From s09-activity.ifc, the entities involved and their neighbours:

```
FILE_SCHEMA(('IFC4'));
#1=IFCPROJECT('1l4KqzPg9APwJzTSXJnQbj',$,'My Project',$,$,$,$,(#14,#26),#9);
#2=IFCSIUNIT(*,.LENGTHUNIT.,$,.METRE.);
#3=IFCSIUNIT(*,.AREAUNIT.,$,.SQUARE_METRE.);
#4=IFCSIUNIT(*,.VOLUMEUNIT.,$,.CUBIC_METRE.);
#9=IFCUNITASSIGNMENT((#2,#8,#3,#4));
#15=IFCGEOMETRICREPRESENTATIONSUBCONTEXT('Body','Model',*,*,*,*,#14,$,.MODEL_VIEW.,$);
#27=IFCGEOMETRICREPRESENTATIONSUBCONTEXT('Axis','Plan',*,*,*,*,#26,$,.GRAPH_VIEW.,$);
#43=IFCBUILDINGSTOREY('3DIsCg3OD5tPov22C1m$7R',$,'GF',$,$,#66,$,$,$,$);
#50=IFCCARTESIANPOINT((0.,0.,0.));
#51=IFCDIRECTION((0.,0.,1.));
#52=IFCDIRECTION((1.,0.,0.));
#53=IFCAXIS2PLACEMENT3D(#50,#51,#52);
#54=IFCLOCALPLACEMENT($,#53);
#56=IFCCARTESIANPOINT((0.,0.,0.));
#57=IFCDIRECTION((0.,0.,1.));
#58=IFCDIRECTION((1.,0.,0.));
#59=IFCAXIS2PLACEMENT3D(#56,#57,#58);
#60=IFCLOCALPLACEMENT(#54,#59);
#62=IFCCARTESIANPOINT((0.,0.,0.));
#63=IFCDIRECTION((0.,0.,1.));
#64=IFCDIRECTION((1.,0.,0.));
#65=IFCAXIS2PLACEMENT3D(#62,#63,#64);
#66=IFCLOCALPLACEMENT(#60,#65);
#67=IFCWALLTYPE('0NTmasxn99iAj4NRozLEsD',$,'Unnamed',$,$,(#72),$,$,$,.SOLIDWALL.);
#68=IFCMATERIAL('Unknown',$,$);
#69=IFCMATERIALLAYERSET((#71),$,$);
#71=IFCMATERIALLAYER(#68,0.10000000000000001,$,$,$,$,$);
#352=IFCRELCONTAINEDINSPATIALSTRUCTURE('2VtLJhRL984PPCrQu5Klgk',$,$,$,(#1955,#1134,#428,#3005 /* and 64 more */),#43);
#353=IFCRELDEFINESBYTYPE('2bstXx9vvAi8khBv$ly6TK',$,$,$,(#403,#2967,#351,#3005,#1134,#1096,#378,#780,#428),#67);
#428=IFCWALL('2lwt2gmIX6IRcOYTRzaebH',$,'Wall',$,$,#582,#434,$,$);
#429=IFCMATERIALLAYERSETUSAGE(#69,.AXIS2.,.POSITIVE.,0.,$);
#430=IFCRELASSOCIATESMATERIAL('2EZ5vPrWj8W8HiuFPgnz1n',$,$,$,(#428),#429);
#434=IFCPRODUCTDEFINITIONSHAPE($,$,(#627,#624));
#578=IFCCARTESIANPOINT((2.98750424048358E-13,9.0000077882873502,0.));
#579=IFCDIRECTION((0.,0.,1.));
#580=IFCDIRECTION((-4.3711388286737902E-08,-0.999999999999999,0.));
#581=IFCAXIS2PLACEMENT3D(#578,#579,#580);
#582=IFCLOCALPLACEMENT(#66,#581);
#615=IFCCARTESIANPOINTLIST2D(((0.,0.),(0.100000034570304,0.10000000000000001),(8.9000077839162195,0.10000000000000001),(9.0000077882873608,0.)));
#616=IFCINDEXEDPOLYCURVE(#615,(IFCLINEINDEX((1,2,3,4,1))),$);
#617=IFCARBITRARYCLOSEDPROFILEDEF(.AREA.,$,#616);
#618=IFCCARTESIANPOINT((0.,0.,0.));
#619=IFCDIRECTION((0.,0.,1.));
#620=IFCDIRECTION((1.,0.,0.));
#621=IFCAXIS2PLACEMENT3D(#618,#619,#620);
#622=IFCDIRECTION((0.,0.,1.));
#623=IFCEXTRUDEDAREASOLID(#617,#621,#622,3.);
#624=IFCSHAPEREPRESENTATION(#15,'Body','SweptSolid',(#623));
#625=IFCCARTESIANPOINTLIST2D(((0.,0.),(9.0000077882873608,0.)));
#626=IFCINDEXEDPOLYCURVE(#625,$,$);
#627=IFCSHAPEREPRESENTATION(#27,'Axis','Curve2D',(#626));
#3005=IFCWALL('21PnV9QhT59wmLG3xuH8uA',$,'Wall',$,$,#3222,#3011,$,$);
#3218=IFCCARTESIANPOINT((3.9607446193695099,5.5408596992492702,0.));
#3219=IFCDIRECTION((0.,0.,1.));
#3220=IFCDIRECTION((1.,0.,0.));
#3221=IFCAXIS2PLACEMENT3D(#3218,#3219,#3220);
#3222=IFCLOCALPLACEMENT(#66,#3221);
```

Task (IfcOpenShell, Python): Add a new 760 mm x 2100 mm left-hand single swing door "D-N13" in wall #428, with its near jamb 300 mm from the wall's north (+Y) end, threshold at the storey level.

```python
import numpy as np
import ifcopenshell
import ifcopenshell.api.feature
import ifcopenshell.api.geometry
import ifcopenshell.api.root
import ifcopenshell.api.spatial
import ifcopenshell.geom
import ifcopenshell.util.element
import ifcopenshell.util.placement
import ifcopenshell.util.representation
import ifcopenshell.util.shape
import ifcopenshell.util.unit

model = ifcopenshell.open("s09-activity.ifc")
unit_scale = ifcopenshell.util.unit.calculate_unit_scale(model)
settings = ifcopenshell.geom.settings()


def volume(element):
    """Net volume in cubic metres, openings subtracted."""
    shape = ifcopenshell.geom.create_shape(settings, element)
    return ifcopenshell.util.shape.get_volume(shape.geometry)


wall = model.by_guid("2lwt2gmIX6IRcOYTRzaebH")
storey = ifcopenshell.util.element.get_container(wall, ifc_class="IfcBuildingStorey")
context = ifcopenshell.util.representation.get_context(model, "Model", "Body", "MODEL_VIEW")
before = volume(wall)

width, height, from_end, sill = 0.76, 2.1, 0.3, 0.0  # metres

# The wall runs along its own X axis, and the end named is its -X end.
wall_shape = ifcopenshell.geom.create_shape(settings, wall)
x, y, z = ifcopenshell.util.shape.get_vertices(wall_shape.geometry).T
start = x.min() + from_end
face, thickness = float(y.min()), float(y.max() - y.min())
wall_matrix = ifcopenshell.util.placement.get_local_placement(wall.ObjectPlacement)
level = ifcopenshell.util.placement.get_local_placement(storey.ObjectPlacement)[2, 3]


def in_wall(x, y):
    """Placement at x, y metres in the wall's axes, at sill height."""
    matrix = wall_matrix.copy()
    matrix[:, 3] = wall_matrix @ np.array([x / unit_scale, y / unit_scale, 0.0, 1.0])
    matrix[2, 3] = level + sill / unit_scale
    return matrix


# Opening: a box that overshoots both wall faces by 50 mm.
opening = ifcopenshell.api.root.create_entity(model, ifc_class="IfcOpeningElement", predefined_type="OPENING")
box = ifcopenshell.api.geometry.add_wall_representation(
    model, context=context, length=width, height=height, thickness=thickness + 0.1
)
ifcopenshell.api.geometry.assign_representation(model, product=opening, representation=box)
ifcopenshell.api.geometry.edit_object_placement(model, product=opening, matrix=in_wall(start, face - 0.05), is_si=False)
ifcopenshell.api.feature.add_feature(model, feature=opening, element=wall)

door = ifcopenshell.api.root.create_entity(model, ifc_class="IfcDoor", name="D-N13", predefined_type="DOOR")
door.OverallWidth, door.OverallHeight = width / unit_scale, height / unit_scale
door.OperationType = "SINGLE_SWING_LEFT"
body = ifcopenshell.api.geometry.add_door_representation(
    model,
    context=context,
    overall_width=door.OverallWidth,
    overall_height=door.OverallHeight,
    operation_type="SINGLE_SWING_LEFT",
    lining_properties={"LiningDepth": thickness / unit_scale, "ThresholdDepth": thickness / unit_scale},
)
ifcopenshell.api.geometry.assign_representation(model, product=door, representation=body)
ifcopenshell.api.spatial.assign_container(model, products=[door], relating_structure=storey)
ifcopenshell.api.feature.add_filling(model, opening=opening, element=door)

# The lining spans the wall, so the door starts at the wall face.
ifcopenshell.api.geometry.edit_object_placement(model, product=door, matrix=in_wall(start, face), is_si=False)

after = volume(wall)

print(f"wall volume {before:.3f} -> {after:.3f} m3")

model.write("s09-activity-out.ifc")
```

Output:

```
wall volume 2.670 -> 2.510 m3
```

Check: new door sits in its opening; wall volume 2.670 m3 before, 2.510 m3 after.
